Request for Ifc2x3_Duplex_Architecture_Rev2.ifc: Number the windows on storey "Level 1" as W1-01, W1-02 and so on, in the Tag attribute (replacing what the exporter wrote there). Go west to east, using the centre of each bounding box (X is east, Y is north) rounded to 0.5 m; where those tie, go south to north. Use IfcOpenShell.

First a look at what the model holds.

```python
import ifcopenshell
import ifcopenshell.util.element
import ifcopenshell.util.placement

model = ifcopenshell.open("Ifc2x3_Duplex_Architecture_Rev2.ifc")
print(model.schema)
storey = next(s for s in model.by_type("IfcBuildingStorey") if s.Name == "Level 1")
windows = [e for e in ifcopenshell.util.element.get_decomposition(storey) if e.is_a("IfcWindow")]
for e in sorted(windows, key=lambda e: e.id()):
    origin = ifcopenshell.util.placement.get_local_placement(e.ObjectPlacement)[:3, 3]
    print(e.id(), e.Tag, e.Name, origin.round(2) + 0.0, sep=" | ")
```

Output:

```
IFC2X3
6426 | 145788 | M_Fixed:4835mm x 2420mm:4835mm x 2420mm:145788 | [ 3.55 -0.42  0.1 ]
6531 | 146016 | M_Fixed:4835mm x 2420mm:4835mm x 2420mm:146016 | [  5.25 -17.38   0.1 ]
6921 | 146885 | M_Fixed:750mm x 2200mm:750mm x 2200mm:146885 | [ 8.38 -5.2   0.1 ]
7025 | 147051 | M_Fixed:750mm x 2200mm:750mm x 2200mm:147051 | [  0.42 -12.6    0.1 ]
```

```python
import ifcopenshell
import ifcopenshell.geom
import ifcopenshell.util.element
import ifcopenshell.util.shape

model = ifcopenshell.open("Ifc2x3_Duplex_Architecture_Rev2.ifc")
settings = ifcopenshell.geom.settings()
settings.set("use-world-coords", True)


def centre(element):
    shape = ifcopenshell.geom.create_shape(settings, element)
    return ifcopenshell.util.shape.get_bbox_centroid(shape.geometry)


storey = next(s for s in model.by_type("IfcBuildingStorey") if s.Name == "Level 1")
windows = [e for e in ifcopenshell.util.element.get_decomposition(storey) if e.is_a("IfcWindow")]

# Insertion points can sit at a corner or the storey origin, so sort by the geometry (in metres).
centres = {e: centre(e) for e in windows}
windows.sort(key=lambda e: (round(centres[e][0] / 0.5), centres[e][1]))

for i, e in enumerate(windows, start=1):
    number = f"W1-{i:02d}"
    e.Tag = number
    print(e.id(), number)

model.write("Ifc2x3_Duplex_Architecture_Rev2_v2.ifc")
```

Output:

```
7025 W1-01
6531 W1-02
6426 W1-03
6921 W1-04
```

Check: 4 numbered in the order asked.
